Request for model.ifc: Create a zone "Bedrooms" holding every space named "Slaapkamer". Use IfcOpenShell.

First a look at what the model holds.

```python
import ifcopenshell

model = ifcopenshell.open("model.ifc")
print(model.schema)
seen = {}
for space in model.by_type("IfcSpace"):
    seen[space.LongName] = seen.get(space.LongName, 0) + 1
for name, count in sorted(seen.items(), key=str):
    print(count, "x", name)
print("zones:", [z.Name for z in model.by_type("IfcZone")][:20])
```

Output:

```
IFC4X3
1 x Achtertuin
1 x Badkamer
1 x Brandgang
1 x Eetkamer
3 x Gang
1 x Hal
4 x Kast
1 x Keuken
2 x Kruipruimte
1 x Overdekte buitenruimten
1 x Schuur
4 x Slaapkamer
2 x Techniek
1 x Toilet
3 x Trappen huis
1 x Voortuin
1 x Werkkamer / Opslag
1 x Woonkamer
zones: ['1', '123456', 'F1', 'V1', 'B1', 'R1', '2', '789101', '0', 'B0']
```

```python
import ifcopenshell
import ifcopenshell.api.group
import ifcopenshell.api.root

model = ifcopenshell.open("model.ifc")

names = {"Slaapkamer"}
spaces = [s for s in model.by_type("IfcSpace") if s.LongName in names]

zone = ifcopenshell.api.root.create_entity(model, ifc_class="IfcZone", name="Bedrooms")
ifcopenshell.api.group.assign_group(model, products=spaces, group=zone)
print(len(spaces), "spaces in", zone.Name)

model.write("model_v2.ifc")
```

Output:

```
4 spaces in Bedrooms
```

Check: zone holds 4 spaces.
